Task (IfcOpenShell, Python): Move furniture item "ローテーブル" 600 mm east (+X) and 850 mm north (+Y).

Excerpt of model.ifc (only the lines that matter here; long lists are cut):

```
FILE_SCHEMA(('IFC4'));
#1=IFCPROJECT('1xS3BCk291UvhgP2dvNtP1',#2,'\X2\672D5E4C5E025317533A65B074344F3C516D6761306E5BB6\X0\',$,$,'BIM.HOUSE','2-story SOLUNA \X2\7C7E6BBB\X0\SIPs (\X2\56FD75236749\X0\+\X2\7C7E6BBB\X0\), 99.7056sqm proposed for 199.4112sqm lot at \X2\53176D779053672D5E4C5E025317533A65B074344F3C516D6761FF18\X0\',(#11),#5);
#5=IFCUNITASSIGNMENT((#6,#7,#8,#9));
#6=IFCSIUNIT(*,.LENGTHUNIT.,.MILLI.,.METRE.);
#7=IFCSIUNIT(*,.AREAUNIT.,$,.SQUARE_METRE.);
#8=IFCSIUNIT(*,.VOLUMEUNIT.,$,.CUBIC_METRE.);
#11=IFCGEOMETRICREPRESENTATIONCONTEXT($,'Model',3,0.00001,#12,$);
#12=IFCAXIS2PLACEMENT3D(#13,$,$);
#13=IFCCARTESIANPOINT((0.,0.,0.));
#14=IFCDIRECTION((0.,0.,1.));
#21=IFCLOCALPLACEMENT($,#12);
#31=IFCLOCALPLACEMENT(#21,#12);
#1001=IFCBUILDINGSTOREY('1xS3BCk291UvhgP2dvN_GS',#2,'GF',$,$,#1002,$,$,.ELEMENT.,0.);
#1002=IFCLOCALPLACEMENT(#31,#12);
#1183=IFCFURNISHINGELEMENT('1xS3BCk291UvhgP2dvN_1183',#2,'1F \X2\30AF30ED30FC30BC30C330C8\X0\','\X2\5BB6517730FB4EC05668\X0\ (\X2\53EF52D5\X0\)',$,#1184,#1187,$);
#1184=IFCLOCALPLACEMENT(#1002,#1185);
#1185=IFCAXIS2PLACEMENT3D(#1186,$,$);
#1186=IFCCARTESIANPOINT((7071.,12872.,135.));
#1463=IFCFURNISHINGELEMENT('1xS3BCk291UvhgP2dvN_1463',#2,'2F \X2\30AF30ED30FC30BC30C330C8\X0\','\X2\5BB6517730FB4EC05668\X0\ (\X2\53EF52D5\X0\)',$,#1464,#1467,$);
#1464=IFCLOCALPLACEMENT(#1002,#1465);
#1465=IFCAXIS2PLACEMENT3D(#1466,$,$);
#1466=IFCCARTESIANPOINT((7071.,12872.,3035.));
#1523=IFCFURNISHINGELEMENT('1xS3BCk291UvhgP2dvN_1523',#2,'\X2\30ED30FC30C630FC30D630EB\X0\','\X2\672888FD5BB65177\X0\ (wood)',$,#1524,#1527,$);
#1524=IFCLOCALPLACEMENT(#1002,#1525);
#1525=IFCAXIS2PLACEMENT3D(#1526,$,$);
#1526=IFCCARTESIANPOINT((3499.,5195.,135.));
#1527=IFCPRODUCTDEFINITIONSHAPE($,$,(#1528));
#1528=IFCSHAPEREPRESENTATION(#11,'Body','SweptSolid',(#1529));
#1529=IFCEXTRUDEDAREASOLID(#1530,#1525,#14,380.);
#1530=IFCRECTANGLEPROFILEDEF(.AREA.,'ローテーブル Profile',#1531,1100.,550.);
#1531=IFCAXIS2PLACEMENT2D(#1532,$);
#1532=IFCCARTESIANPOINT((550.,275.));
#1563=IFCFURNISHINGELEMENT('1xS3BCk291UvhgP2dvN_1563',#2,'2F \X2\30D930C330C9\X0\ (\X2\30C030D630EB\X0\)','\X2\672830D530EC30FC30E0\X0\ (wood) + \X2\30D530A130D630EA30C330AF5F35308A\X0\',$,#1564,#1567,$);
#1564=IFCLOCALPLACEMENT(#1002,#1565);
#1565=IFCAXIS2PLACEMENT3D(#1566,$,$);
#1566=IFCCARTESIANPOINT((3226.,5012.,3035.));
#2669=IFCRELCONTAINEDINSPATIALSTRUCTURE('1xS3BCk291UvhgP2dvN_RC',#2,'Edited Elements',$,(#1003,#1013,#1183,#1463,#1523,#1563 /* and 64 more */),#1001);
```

```python
import ifcopenshell
import ifcopenshell.api.geometry
import ifcopenshell.util.placement
import ifcopenshell.util.unit

model = ifcopenshell.open("model.ifc")
unit_scale = ifcopenshell.util.unit.calculate_unit_scale(model)

item = model.by_id(1523)
matrix = ifcopenshell.util.placement.get_local_placement(item.ObjectPlacement)
matrix[0, 3] += 0.6 / unit_scale
matrix[1, 3] += 0.85 / unit_scale
ifcopenshell.api.geometry.edit_object_placement(model, product=item, matrix=matrix, is_si=False)

print(ifcopenshell.util.placement.get_local_placement(item.ObjectPlacement).round(3) + 0.0)

model.write("model_updated.ifc")
```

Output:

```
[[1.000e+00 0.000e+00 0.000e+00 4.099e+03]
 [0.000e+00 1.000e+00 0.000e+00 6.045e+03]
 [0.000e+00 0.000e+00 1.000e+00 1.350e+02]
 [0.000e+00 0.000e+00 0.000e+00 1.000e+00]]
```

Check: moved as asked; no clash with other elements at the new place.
